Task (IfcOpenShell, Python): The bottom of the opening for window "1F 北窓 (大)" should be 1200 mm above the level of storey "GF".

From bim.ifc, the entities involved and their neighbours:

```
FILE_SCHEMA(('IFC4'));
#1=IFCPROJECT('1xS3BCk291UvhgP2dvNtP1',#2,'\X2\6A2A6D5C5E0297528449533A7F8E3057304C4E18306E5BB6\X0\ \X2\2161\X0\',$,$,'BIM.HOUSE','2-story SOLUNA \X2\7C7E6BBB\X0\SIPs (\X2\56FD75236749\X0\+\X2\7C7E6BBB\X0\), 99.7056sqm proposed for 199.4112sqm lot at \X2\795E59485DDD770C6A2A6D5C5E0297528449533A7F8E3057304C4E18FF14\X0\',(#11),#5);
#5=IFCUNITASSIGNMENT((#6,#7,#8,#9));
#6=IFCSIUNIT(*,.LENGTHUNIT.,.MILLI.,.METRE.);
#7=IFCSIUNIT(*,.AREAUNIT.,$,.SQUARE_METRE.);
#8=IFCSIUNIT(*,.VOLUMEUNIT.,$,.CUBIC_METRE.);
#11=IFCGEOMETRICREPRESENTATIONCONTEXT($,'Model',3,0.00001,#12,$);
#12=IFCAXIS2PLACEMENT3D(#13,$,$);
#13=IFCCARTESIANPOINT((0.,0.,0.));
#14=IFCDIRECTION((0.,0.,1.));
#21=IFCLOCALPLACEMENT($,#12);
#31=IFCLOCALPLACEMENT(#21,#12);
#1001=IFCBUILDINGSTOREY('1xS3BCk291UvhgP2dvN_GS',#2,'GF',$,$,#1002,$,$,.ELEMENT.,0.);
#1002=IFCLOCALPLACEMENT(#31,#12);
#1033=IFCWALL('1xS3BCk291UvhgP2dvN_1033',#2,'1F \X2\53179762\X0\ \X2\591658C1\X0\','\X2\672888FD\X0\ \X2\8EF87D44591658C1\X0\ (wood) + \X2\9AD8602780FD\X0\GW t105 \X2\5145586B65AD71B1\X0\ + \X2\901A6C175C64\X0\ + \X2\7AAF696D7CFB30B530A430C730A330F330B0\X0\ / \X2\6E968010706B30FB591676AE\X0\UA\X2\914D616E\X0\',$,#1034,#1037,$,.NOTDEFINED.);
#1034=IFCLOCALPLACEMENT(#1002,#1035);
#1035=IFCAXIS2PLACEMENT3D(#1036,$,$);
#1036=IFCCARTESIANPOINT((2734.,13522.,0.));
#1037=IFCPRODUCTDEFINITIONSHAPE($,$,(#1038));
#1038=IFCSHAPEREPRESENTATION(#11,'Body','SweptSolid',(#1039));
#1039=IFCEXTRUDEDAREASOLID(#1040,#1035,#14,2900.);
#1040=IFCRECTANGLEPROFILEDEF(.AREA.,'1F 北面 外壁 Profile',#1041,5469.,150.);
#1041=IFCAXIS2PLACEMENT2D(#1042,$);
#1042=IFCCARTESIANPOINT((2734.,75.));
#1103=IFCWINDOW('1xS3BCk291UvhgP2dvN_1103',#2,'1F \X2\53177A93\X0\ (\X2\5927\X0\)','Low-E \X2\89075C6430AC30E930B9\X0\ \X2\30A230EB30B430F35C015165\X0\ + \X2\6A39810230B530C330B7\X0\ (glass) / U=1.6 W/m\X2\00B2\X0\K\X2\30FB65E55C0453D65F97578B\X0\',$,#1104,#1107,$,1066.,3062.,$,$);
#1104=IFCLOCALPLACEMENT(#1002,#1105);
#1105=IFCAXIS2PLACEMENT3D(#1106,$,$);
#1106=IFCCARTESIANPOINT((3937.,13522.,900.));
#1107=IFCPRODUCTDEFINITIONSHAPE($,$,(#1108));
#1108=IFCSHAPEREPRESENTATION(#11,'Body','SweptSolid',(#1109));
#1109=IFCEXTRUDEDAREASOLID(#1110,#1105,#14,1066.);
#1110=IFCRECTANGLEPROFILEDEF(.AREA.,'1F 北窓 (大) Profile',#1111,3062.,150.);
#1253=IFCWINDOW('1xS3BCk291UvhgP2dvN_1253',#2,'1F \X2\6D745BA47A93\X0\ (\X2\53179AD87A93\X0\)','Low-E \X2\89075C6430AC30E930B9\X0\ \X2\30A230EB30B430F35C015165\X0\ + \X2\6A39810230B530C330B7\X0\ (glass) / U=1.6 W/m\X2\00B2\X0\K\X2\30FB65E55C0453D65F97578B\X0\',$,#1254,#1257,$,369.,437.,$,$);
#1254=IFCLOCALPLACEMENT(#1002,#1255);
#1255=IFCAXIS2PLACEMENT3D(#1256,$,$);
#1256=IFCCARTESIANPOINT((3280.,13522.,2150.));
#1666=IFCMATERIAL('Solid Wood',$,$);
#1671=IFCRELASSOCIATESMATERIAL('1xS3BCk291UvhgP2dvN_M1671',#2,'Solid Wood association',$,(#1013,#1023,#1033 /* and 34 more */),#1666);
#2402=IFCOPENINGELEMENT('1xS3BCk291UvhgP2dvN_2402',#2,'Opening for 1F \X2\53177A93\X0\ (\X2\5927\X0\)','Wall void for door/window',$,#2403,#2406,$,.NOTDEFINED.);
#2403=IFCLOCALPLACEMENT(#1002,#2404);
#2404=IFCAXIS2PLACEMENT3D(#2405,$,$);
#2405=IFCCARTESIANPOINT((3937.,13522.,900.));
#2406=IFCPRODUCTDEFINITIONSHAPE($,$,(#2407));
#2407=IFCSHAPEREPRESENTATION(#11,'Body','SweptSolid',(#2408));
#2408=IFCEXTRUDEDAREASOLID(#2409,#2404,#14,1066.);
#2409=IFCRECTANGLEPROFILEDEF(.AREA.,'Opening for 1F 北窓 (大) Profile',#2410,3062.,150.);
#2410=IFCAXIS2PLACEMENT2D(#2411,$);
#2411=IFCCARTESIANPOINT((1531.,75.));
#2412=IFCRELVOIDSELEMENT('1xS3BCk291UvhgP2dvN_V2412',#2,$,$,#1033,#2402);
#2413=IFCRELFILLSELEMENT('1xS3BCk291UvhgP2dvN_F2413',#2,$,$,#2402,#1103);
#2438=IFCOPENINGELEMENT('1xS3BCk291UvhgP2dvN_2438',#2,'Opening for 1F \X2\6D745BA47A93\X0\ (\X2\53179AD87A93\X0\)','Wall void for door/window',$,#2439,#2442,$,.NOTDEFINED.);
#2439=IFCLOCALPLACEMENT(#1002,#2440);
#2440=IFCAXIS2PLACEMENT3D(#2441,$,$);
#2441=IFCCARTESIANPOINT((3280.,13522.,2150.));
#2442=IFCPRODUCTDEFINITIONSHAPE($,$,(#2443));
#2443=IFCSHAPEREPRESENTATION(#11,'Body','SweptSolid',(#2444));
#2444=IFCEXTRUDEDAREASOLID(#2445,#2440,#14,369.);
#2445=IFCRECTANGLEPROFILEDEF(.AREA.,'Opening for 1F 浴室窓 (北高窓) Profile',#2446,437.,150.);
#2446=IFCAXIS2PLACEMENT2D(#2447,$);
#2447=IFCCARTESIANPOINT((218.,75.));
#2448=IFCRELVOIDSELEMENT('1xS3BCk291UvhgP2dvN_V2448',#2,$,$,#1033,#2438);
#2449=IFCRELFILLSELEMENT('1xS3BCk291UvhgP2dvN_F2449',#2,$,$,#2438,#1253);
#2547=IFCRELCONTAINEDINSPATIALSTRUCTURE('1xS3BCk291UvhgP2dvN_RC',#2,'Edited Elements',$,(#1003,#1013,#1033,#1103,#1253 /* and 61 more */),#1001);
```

```python
import numpy as np
import ifcopenshell
import ifcopenshell.api.geometry
import ifcopenshell.geom
import ifcopenshell.util.element
import ifcopenshell.util.placement
import ifcopenshell.util.shape
import ifcopenshell.util.unit

model = ifcopenshell.open("bim.ifc")
unit_scale = ifcopenshell.util.unit.calculate_unit_scale(model)

window = model.by_guid("1xS3BCk291UvhgP2dvN_1103")
opening = window.FillsVoids[0].RelatingOpeningElement
storey = ifcopenshell.util.element.get_container(window, ifc_class="IfcBuildingStorey")
level = ifcopenshell.util.placement.get_local_placement(storey.ObjectPlacement)[2, 3]

# The opening's origin need not be at the sill, so measure its lowest point.
shape = ifcopenshell.geom.create_shape(ifcopenshell.geom.settings(), opening)
bottom = ifcopenshell.util.shape.get_shape_bottom_elevation(shape, shape.geometry) / unit_scale
dz = level + 1.2 / unit_scale - bottom

shift = np.array([0.0, 0.0, dz])
# The window is not placed relative to its opening, so move both.
for product in (opening, window):
    matrix = ifcopenshell.util.placement.get_local_placement(product.ObjectPlacement)
    matrix[:3, 3] += shift
    ifcopenshell.api.geometry.edit_object_placement(model, product=product, matrix=matrix, is_si=False)

print(f"moved by {dz * unit_scale:+.3f} m")

model.write("bim_rev.ifc")
```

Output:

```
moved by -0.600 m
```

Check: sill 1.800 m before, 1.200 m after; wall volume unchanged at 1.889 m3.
